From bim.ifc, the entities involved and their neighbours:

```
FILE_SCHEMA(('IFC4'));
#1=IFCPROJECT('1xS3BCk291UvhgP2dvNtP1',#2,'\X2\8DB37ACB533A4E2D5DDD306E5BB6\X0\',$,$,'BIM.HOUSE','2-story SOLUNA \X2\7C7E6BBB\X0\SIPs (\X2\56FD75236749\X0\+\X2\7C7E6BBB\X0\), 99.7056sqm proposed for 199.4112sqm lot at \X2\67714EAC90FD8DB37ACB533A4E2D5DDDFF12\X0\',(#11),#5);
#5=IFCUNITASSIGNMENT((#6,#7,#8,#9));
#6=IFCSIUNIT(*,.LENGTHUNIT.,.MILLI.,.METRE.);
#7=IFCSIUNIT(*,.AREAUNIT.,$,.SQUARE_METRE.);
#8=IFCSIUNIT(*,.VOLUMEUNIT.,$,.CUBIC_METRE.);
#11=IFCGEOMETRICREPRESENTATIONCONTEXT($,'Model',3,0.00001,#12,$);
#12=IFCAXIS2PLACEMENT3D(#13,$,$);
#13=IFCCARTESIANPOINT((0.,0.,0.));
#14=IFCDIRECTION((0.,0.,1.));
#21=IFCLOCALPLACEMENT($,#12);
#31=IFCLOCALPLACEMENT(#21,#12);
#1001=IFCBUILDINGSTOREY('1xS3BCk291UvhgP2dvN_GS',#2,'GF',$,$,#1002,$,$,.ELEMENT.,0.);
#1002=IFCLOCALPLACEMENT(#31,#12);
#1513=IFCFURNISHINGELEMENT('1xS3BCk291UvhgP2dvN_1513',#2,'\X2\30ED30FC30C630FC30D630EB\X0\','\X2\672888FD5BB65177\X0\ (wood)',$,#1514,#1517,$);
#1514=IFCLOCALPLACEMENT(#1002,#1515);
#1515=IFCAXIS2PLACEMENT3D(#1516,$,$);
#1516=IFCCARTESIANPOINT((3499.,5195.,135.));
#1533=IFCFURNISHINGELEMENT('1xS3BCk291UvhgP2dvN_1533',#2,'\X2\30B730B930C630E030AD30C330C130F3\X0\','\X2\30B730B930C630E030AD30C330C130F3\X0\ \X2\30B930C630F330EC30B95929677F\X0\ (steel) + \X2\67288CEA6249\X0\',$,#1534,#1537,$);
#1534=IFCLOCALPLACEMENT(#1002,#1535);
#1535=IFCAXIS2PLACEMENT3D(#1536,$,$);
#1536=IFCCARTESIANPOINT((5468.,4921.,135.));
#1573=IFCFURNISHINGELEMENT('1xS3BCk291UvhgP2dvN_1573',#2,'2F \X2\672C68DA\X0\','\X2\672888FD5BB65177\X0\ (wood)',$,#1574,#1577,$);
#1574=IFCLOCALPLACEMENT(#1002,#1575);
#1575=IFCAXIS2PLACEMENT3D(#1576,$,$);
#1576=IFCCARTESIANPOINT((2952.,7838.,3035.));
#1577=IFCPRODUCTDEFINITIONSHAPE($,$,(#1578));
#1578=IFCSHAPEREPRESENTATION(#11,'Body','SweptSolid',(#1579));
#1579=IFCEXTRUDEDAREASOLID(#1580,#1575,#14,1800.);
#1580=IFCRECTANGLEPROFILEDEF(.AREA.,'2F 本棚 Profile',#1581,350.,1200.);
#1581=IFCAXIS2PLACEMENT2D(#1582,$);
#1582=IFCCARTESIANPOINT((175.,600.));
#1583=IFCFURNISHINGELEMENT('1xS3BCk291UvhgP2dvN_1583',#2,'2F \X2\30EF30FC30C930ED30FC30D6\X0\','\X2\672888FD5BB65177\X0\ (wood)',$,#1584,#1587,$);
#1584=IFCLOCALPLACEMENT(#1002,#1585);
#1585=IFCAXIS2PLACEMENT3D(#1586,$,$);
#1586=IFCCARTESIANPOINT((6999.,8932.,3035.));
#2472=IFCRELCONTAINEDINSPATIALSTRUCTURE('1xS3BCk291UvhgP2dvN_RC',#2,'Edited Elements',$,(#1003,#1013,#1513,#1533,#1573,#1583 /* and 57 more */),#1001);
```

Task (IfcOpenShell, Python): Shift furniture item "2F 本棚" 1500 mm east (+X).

```python
import ifcopenshell
import ifcopenshell.api.geometry
import ifcopenshell.util.placement
import ifcopenshell.util.unit

model = ifcopenshell.open("bim.ifc")
unit_scale = ifcopenshell.util.unit.calculate_unit_scale(model)

item = model.by_guid("1xS3BCk291UvhgP2dvN_1573")
matrix = ifcopenshell.util.placement.get_local_placement(item.ObjectPlacement)
matrix[0, 3] += 1.5 / unit_scale
ifcopenshell.api.geometry.edit_object_placement(model, product=item, matrix=matrix, is_si=False)

print(ifcopenshell.util.placement.get_local_placement(item.ObjectPlacement).round(3) + 0.0)

model.write("bim-out.ifc")
```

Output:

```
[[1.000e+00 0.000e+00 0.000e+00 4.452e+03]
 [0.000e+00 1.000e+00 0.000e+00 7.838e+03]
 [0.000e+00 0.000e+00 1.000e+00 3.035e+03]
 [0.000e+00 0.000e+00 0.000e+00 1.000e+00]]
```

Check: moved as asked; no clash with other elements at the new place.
